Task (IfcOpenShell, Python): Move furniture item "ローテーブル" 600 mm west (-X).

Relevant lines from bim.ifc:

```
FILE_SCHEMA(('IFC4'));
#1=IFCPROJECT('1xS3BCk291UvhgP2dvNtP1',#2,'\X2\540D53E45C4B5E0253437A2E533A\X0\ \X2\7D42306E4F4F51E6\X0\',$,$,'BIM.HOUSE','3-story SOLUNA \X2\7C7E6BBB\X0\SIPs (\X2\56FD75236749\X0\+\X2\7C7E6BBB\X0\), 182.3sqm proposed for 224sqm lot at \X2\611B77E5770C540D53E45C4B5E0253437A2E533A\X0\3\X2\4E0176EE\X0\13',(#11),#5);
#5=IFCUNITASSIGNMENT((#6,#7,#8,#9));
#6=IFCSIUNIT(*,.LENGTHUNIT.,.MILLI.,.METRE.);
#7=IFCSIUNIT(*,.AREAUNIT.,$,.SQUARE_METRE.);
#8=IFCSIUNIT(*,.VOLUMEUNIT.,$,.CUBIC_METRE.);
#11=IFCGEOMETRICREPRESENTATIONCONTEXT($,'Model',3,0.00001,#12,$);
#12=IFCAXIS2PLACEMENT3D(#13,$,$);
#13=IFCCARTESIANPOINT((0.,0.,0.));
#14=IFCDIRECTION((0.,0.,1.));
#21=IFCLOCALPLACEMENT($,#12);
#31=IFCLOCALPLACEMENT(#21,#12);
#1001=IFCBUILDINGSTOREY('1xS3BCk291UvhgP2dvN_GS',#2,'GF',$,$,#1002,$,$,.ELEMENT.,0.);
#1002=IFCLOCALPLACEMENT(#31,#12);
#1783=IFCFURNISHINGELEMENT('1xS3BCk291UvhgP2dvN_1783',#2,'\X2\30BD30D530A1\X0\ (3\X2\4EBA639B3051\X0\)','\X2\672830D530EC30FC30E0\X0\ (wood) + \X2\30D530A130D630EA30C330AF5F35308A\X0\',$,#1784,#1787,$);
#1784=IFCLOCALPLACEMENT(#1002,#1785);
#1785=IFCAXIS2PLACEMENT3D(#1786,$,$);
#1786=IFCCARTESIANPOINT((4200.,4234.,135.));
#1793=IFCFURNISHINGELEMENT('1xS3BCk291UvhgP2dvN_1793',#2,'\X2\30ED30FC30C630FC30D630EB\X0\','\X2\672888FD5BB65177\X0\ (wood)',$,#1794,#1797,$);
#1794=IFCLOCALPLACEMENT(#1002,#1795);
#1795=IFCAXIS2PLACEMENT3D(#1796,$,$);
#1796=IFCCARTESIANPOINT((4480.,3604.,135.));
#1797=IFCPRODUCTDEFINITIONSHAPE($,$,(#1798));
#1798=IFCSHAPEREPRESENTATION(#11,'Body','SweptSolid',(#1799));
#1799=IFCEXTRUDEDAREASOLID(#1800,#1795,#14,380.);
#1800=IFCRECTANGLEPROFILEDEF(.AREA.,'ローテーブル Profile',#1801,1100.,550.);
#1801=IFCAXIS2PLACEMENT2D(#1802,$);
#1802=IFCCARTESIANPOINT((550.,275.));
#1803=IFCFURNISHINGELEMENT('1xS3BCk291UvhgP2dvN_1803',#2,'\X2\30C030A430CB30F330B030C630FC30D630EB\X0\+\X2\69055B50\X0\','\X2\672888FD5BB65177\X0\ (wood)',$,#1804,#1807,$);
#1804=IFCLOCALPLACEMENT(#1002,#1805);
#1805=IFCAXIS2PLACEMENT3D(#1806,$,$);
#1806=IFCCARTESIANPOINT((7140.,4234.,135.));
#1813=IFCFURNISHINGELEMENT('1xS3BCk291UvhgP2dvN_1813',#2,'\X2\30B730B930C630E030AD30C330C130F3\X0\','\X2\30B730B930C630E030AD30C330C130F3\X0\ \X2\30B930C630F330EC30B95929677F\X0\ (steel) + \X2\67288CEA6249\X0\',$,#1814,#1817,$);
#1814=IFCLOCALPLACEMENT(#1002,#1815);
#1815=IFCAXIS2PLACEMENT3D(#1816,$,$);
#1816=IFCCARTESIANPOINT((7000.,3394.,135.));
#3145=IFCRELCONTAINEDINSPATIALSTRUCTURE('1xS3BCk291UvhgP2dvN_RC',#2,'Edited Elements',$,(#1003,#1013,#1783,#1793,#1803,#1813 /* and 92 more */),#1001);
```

```python
import ifcopenshell
import ifcopenshell.api.geometry
import ifcopenshell.util.placement

model = ifcopenshell.open("bim.ifc")

item = model.by_id(1793)
matrix = ifcopenshell.util.placement.get_local_placement(item.ObjectPlacement)
matrix[0, 3] -= 600.0
ifcopenshell.api.geometry.edit_object_placement(model, product=item, matrix=matrix, is_si=False)

print(ifcopenshell.util.placement.get_local_placement(item.ObjectPlacement).round(3) + 0.0)

model.write("bim_v2.ifc")
```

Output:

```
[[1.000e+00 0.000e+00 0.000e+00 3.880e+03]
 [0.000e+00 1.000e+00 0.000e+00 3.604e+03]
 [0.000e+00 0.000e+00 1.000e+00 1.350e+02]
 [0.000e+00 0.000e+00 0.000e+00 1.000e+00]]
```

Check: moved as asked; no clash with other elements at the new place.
